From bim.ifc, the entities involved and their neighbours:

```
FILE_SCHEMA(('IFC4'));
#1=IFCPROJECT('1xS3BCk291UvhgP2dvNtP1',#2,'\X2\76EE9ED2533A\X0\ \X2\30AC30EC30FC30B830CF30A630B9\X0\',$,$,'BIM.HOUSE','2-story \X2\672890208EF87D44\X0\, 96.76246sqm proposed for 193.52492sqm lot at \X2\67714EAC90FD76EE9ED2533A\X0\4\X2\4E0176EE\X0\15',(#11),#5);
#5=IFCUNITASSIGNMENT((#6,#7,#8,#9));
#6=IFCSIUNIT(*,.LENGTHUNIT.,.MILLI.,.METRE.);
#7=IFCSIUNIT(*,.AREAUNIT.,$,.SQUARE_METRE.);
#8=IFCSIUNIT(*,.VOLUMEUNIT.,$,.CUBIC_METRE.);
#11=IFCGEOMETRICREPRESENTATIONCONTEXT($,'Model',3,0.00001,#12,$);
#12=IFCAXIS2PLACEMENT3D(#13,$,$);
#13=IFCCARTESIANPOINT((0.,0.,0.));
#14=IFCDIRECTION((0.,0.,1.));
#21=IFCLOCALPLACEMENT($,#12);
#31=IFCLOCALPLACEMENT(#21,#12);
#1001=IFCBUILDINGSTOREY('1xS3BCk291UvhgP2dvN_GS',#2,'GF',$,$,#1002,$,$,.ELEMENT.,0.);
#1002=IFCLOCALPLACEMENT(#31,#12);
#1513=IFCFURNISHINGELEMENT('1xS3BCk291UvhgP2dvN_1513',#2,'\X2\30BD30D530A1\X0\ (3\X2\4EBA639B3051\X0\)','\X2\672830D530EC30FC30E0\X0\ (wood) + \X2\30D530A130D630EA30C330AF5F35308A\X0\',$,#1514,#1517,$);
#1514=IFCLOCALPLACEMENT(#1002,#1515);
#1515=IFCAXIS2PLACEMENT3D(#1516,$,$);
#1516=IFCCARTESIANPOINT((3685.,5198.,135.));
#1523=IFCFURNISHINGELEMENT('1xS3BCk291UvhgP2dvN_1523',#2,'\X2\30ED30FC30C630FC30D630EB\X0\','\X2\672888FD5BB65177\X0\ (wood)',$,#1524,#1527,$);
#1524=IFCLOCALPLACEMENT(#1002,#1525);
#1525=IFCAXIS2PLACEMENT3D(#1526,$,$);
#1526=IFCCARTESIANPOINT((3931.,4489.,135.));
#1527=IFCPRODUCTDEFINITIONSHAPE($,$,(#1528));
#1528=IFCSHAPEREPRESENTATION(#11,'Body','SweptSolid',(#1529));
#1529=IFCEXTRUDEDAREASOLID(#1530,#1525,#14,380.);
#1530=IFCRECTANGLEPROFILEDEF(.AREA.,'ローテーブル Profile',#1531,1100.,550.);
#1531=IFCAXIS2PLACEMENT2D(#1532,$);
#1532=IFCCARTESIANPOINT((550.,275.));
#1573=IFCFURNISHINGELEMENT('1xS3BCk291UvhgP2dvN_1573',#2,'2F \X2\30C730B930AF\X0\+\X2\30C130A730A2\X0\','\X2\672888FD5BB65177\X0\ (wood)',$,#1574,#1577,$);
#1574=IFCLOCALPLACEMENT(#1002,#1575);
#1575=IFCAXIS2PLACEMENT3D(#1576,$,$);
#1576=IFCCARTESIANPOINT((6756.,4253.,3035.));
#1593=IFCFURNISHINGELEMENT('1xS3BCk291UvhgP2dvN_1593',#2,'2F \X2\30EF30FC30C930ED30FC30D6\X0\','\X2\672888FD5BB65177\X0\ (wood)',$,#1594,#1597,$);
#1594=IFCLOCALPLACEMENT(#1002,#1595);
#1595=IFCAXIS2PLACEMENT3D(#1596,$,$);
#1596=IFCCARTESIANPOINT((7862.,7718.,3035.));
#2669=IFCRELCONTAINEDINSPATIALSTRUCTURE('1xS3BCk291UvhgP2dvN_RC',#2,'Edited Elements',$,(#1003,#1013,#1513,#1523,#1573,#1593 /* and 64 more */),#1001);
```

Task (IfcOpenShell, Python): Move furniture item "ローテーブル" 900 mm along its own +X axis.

```python
import ifcopenshell
import ifcopenshell.api.geometry
import ifcopenshell.util.placement
import ifcopenshell.util.unit

model = ifcopenshell.open("bim.ifc")
unit_scale = ifcopenshell.util.unit.calculate_unit_scale(model)

item = model.by_guid("1xS3BCk291UvhgP2dvN_1523")
matrix = ifcopenshell.util.placement.get_local_placement(item.ObjectPlacement)
matrix[:3, 3] += matrix[:3, 0] * 0.9 / unit_scale
ifcopenshell.api.geometry.edit_object_placement(model, product=item, matrix=matrix, is_si=False)

print(ifcopenshell.util.placement.get_local_placement(item.ObjectPlacement).round(3) + 0.0)

model.write("bim-out.ifc")
```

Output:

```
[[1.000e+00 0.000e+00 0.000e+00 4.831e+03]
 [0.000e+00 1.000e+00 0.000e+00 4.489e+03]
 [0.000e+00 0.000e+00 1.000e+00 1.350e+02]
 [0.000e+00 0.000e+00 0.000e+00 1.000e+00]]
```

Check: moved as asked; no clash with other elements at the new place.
